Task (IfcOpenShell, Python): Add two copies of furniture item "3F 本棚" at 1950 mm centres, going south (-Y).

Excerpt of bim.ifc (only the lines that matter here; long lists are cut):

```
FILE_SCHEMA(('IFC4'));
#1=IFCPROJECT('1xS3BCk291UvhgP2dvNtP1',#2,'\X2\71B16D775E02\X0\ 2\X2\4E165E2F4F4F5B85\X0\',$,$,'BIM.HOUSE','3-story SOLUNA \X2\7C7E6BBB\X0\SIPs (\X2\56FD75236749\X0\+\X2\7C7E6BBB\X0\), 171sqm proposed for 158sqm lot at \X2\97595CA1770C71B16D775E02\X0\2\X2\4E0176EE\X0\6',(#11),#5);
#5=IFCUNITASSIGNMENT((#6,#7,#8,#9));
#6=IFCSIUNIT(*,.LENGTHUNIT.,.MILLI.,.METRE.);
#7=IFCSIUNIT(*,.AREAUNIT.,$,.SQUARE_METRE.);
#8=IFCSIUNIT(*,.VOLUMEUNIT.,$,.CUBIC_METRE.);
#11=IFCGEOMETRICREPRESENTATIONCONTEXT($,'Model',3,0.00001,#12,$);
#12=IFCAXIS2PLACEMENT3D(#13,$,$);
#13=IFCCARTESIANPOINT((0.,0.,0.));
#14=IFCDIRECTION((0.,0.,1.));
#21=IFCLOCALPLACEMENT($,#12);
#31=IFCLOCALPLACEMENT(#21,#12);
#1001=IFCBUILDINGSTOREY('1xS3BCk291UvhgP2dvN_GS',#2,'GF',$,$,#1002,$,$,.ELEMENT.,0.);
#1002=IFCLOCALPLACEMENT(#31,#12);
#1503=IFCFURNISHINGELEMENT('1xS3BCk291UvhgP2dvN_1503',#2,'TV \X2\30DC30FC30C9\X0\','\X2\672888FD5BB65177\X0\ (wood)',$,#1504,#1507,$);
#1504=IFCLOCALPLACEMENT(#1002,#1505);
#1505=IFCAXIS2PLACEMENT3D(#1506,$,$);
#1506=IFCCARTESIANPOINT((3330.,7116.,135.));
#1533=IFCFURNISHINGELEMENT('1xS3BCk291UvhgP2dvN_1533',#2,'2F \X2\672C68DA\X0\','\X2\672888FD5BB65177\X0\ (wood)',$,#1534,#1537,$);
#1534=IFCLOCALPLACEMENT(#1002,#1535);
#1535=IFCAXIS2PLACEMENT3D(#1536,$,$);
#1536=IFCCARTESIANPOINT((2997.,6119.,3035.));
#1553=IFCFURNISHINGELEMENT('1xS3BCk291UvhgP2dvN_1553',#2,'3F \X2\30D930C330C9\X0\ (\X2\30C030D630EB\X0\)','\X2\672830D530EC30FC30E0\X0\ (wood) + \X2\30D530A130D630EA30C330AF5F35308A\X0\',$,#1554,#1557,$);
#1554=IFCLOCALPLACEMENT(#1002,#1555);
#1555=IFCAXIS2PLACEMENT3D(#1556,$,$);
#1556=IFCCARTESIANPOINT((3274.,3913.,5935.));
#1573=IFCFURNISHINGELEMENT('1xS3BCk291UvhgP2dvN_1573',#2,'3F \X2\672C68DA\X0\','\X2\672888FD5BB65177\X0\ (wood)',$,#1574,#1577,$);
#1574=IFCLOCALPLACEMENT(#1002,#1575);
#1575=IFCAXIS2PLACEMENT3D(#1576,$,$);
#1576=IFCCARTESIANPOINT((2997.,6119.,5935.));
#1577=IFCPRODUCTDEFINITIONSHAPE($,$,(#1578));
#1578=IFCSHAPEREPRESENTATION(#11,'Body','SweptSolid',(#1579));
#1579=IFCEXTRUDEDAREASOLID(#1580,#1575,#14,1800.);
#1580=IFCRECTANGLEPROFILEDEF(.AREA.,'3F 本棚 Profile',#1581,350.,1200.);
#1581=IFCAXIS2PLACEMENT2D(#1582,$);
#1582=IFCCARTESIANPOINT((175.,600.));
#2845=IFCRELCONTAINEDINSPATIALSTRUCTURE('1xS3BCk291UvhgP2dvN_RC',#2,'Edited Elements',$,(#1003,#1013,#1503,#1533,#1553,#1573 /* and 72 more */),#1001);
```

```python
import numpy as np
import ifcopenshell
import ifcopenshell.api.geometry
import ifcopenshell.api.root
import ifcopenshell.util.element
import ifcopenshell.util.placement

model = ifcopenshell.open("bim.ifc")


def reuse_history(source, copy):
    """copy_class also copies each property set's owner history, people and application; keep the originals."""
    for rel in copy.IsDefinedBy:
        if rel.is_a("IfcRelDefinesByProperties") and (history := rel.RelatingPropertyDefinition.OwnerHistory):
            rel.RelatingPropertyDefinition.OwnerHistory = source.OwnerHistory
            ifcopenshell.util.element.remove_deep2(model, history)


source = model.by_id(1573)
base = ifcopenshell.util.placement.get_local_placement(source.ObjectPlacement)
step = np.array([0.0, -1.0, 0.0]) * 1950.0

for i in range(1, 3):
    copy = ifcopenshell.api.root.copy_class(model, product=source)
    copy.Representation = ifcopenshell.util.element.copy_deep(
        model, source.Representation, exclude=["IfcGeometricRepresentationContext", "IfcRepresentationMap"]
    )
    reuse_history(source, copy)
    matrix = base.copy()
    matrix[:3, 3] += i * step
    print("added at", matrix[:3, 3].round(3) + 0.0)
    ifcopenshell.api.geometry.edit_object_placement(model, product=copy, matrix=matrix, is_si=False)

model.write("bim_edited.ifc")
```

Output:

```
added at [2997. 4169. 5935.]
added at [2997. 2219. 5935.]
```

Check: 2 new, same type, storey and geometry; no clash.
